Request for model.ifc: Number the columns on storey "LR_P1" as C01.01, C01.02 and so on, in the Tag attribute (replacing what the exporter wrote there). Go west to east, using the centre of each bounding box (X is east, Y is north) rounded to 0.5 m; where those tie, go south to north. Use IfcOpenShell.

First a look at what the model holds.

```python
import ifcopenshell
import ifcopenshell.util.element
import ifcopenshell.util.placement

model = ifcopenshell.open("model.ifc")
print(model.schema)
storey = next(s for s in model.by_type("IfcBuildingStorey") if s.Name == "LR_P1")
columns = [e for e in ifcopenshell.util.element.get_decomposition(storey) if e.is_a("IfcColumn")]
for e in sorted(columns, key=lambda e: e.id()):
    origin = ifcopenshell.util.placement.get_local_placement(e.ObjectPlacement)[:3, 3]
    print(e.id(), e.Tag, e.Name, origin.round(2) + 0.0, sep=" | ")
```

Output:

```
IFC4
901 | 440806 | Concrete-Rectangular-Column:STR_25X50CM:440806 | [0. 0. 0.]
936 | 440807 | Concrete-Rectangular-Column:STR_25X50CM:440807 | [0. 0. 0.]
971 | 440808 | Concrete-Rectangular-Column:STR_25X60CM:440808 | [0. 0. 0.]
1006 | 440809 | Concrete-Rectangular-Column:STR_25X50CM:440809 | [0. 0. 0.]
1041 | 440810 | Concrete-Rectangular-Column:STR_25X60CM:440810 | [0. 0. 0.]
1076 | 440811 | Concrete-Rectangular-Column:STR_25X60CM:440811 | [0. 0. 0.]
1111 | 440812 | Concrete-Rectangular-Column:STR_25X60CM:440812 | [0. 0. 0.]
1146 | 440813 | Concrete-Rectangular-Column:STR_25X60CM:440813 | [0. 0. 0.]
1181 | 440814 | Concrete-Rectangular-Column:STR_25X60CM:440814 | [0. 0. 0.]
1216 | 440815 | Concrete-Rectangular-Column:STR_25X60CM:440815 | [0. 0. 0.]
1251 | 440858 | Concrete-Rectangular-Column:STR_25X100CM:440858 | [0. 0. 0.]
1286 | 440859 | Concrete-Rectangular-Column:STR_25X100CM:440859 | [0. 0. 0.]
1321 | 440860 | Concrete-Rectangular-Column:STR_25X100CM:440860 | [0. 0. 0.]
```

```python
import ifcopenshell
import ifcopenshell.geom
import ifcopenshell.util.element
import ifcopenshell.util.shape

model = ifcopenshell.open("model.ifc")
settings = ifcopenshell.geom.settings()
settings.set("use-world-coords", True)


def centre(element):
    shape = ifcopenshell.geom.create_shape(settings, element)
    return ifcopenshell.util.shape.get_bbox_centroid(shape.geometry)


storey = next(s for s in model.by_type("IfcBuildingStorey") if s.Name == "LR_P1")
columns = [e for e in ifcopenshell.util.element.get_decomposition(storey) if e.is_a("IfcColumn")]

# Insertion points can sit at a corner or the storey origin, so sort by the geometry (in metres).
centres = {e: centre(e) for e in columns}
columns.sort(key=lambda e: (round(centres[e][0] / 0.5), centres[e][1]))

for i, e in enumerate(columns, start=1):
    number = f"C01.{i:02d}"
    e.Tag = number
    print(e.id(), number)

model.write("model-out.ifc")
```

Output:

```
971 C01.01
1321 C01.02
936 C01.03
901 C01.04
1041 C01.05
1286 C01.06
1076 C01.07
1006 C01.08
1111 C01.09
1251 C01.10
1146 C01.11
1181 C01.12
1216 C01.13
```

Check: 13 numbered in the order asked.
